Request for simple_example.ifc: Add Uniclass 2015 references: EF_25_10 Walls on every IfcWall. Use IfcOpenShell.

First a look at what the model holds.

```python
import ifcopenshell

model = ifcopenshell.open("simple_example.ifc")
print(model.schema)
print("classifications:", [c.Name for c in model.by_type("IfcClassification")])
for ifc_class in ("IfcDoor", "IfcRoof", "IfcStair", "IfcWall", "IfcWindow"):
    print(ifc_class, len(model.by_type(ifc_class)))
```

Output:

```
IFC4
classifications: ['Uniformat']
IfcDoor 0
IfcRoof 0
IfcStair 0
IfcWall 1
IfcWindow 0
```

```python
import ifcopenshell
import ifcopenshell.api.classification

model = ifcopenshell.open("simple_example.ifc")

system = ifcopenshell.api.classification.add_classification(model, classification="Uniclass 2015")

codes = {
    "IfcWall": ("EF_25_10", "Walls"),
}
for ifc_class, (code, name) in codes.items():
    products = model.by_type(ifc_class)
    ifcopenshell.api.classification.add_reference(
        model, products=products, classification=system, identification=code, name=name
    )
    print(code, len(products))

model.write("simple_example_v2.ifc")
```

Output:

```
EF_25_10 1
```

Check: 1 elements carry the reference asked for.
